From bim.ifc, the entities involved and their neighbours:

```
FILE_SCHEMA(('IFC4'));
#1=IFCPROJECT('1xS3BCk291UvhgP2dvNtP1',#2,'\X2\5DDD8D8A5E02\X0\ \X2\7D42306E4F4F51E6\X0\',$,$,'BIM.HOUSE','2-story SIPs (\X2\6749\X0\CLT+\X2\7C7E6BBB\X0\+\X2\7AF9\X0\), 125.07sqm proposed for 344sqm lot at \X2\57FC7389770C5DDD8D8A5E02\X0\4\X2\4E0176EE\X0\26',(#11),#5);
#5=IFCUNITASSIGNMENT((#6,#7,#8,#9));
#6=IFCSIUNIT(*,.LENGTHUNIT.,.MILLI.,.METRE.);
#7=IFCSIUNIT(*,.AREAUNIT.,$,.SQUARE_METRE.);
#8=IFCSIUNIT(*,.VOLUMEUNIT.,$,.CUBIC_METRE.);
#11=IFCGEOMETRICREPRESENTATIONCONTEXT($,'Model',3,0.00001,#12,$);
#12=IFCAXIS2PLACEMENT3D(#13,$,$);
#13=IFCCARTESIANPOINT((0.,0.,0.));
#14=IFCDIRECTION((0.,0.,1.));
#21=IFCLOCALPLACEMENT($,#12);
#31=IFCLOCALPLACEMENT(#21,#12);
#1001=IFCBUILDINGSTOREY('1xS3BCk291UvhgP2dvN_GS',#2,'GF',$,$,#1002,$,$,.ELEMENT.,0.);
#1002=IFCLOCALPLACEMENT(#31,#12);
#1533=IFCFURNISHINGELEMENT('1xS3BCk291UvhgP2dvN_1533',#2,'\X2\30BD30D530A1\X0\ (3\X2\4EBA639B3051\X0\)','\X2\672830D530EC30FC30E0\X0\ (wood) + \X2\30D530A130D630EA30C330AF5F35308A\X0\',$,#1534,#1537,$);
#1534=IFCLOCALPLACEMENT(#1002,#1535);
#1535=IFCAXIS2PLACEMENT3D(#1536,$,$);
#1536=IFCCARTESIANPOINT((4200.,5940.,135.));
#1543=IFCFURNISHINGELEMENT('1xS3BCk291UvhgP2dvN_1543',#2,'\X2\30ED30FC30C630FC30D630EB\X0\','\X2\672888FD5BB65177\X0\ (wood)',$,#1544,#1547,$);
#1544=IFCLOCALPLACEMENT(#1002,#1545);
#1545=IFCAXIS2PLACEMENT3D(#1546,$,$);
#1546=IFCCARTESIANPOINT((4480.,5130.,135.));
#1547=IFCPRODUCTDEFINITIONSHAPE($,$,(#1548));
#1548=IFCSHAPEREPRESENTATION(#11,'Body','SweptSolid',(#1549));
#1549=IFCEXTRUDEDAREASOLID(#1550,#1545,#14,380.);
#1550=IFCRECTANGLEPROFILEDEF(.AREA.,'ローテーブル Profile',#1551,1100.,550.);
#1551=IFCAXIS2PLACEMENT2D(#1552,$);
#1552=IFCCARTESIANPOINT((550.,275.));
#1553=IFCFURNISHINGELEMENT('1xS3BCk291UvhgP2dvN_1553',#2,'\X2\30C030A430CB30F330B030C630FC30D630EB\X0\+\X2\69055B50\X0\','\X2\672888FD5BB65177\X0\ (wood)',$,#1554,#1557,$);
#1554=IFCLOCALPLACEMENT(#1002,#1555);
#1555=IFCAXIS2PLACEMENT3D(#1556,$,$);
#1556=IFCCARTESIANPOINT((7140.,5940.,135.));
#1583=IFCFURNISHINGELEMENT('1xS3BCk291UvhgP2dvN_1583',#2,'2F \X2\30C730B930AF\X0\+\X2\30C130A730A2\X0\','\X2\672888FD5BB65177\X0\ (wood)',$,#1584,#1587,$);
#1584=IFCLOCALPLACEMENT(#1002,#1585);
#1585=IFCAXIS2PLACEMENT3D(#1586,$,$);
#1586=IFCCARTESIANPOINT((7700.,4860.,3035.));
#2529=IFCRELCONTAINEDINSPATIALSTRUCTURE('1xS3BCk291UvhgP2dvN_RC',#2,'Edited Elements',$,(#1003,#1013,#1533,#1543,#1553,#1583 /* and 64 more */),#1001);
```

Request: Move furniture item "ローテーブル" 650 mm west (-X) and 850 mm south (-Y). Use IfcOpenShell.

```python
import ifcopenshell
import ifcopenshell.api.geometry
import ifcopenshell.util.placement

model = ifcopenshell.open("bim.ifc")

item = model.by_guid("1xS3BCk291UvhgP2dvN_1543")
matrix = ifcopenshell.util.placement.get_local_placement(item.ObjectPlacement)
matrix[0, 3] -= 650.0
matrix[1, 3] -= 850.0
ifcopenshell.api.geometry.edit_object_placement(model, product=item, matrix=matrix, is_si=False)

print(ifcopenshell.util.placement.get_local_placement(item.ObjectPlacement).round(3) + 0.0)

model.write("bim-out.ifc")
```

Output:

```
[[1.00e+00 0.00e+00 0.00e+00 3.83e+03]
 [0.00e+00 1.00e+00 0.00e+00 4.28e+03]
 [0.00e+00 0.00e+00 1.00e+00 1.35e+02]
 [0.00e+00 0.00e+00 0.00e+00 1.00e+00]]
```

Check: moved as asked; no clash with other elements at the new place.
